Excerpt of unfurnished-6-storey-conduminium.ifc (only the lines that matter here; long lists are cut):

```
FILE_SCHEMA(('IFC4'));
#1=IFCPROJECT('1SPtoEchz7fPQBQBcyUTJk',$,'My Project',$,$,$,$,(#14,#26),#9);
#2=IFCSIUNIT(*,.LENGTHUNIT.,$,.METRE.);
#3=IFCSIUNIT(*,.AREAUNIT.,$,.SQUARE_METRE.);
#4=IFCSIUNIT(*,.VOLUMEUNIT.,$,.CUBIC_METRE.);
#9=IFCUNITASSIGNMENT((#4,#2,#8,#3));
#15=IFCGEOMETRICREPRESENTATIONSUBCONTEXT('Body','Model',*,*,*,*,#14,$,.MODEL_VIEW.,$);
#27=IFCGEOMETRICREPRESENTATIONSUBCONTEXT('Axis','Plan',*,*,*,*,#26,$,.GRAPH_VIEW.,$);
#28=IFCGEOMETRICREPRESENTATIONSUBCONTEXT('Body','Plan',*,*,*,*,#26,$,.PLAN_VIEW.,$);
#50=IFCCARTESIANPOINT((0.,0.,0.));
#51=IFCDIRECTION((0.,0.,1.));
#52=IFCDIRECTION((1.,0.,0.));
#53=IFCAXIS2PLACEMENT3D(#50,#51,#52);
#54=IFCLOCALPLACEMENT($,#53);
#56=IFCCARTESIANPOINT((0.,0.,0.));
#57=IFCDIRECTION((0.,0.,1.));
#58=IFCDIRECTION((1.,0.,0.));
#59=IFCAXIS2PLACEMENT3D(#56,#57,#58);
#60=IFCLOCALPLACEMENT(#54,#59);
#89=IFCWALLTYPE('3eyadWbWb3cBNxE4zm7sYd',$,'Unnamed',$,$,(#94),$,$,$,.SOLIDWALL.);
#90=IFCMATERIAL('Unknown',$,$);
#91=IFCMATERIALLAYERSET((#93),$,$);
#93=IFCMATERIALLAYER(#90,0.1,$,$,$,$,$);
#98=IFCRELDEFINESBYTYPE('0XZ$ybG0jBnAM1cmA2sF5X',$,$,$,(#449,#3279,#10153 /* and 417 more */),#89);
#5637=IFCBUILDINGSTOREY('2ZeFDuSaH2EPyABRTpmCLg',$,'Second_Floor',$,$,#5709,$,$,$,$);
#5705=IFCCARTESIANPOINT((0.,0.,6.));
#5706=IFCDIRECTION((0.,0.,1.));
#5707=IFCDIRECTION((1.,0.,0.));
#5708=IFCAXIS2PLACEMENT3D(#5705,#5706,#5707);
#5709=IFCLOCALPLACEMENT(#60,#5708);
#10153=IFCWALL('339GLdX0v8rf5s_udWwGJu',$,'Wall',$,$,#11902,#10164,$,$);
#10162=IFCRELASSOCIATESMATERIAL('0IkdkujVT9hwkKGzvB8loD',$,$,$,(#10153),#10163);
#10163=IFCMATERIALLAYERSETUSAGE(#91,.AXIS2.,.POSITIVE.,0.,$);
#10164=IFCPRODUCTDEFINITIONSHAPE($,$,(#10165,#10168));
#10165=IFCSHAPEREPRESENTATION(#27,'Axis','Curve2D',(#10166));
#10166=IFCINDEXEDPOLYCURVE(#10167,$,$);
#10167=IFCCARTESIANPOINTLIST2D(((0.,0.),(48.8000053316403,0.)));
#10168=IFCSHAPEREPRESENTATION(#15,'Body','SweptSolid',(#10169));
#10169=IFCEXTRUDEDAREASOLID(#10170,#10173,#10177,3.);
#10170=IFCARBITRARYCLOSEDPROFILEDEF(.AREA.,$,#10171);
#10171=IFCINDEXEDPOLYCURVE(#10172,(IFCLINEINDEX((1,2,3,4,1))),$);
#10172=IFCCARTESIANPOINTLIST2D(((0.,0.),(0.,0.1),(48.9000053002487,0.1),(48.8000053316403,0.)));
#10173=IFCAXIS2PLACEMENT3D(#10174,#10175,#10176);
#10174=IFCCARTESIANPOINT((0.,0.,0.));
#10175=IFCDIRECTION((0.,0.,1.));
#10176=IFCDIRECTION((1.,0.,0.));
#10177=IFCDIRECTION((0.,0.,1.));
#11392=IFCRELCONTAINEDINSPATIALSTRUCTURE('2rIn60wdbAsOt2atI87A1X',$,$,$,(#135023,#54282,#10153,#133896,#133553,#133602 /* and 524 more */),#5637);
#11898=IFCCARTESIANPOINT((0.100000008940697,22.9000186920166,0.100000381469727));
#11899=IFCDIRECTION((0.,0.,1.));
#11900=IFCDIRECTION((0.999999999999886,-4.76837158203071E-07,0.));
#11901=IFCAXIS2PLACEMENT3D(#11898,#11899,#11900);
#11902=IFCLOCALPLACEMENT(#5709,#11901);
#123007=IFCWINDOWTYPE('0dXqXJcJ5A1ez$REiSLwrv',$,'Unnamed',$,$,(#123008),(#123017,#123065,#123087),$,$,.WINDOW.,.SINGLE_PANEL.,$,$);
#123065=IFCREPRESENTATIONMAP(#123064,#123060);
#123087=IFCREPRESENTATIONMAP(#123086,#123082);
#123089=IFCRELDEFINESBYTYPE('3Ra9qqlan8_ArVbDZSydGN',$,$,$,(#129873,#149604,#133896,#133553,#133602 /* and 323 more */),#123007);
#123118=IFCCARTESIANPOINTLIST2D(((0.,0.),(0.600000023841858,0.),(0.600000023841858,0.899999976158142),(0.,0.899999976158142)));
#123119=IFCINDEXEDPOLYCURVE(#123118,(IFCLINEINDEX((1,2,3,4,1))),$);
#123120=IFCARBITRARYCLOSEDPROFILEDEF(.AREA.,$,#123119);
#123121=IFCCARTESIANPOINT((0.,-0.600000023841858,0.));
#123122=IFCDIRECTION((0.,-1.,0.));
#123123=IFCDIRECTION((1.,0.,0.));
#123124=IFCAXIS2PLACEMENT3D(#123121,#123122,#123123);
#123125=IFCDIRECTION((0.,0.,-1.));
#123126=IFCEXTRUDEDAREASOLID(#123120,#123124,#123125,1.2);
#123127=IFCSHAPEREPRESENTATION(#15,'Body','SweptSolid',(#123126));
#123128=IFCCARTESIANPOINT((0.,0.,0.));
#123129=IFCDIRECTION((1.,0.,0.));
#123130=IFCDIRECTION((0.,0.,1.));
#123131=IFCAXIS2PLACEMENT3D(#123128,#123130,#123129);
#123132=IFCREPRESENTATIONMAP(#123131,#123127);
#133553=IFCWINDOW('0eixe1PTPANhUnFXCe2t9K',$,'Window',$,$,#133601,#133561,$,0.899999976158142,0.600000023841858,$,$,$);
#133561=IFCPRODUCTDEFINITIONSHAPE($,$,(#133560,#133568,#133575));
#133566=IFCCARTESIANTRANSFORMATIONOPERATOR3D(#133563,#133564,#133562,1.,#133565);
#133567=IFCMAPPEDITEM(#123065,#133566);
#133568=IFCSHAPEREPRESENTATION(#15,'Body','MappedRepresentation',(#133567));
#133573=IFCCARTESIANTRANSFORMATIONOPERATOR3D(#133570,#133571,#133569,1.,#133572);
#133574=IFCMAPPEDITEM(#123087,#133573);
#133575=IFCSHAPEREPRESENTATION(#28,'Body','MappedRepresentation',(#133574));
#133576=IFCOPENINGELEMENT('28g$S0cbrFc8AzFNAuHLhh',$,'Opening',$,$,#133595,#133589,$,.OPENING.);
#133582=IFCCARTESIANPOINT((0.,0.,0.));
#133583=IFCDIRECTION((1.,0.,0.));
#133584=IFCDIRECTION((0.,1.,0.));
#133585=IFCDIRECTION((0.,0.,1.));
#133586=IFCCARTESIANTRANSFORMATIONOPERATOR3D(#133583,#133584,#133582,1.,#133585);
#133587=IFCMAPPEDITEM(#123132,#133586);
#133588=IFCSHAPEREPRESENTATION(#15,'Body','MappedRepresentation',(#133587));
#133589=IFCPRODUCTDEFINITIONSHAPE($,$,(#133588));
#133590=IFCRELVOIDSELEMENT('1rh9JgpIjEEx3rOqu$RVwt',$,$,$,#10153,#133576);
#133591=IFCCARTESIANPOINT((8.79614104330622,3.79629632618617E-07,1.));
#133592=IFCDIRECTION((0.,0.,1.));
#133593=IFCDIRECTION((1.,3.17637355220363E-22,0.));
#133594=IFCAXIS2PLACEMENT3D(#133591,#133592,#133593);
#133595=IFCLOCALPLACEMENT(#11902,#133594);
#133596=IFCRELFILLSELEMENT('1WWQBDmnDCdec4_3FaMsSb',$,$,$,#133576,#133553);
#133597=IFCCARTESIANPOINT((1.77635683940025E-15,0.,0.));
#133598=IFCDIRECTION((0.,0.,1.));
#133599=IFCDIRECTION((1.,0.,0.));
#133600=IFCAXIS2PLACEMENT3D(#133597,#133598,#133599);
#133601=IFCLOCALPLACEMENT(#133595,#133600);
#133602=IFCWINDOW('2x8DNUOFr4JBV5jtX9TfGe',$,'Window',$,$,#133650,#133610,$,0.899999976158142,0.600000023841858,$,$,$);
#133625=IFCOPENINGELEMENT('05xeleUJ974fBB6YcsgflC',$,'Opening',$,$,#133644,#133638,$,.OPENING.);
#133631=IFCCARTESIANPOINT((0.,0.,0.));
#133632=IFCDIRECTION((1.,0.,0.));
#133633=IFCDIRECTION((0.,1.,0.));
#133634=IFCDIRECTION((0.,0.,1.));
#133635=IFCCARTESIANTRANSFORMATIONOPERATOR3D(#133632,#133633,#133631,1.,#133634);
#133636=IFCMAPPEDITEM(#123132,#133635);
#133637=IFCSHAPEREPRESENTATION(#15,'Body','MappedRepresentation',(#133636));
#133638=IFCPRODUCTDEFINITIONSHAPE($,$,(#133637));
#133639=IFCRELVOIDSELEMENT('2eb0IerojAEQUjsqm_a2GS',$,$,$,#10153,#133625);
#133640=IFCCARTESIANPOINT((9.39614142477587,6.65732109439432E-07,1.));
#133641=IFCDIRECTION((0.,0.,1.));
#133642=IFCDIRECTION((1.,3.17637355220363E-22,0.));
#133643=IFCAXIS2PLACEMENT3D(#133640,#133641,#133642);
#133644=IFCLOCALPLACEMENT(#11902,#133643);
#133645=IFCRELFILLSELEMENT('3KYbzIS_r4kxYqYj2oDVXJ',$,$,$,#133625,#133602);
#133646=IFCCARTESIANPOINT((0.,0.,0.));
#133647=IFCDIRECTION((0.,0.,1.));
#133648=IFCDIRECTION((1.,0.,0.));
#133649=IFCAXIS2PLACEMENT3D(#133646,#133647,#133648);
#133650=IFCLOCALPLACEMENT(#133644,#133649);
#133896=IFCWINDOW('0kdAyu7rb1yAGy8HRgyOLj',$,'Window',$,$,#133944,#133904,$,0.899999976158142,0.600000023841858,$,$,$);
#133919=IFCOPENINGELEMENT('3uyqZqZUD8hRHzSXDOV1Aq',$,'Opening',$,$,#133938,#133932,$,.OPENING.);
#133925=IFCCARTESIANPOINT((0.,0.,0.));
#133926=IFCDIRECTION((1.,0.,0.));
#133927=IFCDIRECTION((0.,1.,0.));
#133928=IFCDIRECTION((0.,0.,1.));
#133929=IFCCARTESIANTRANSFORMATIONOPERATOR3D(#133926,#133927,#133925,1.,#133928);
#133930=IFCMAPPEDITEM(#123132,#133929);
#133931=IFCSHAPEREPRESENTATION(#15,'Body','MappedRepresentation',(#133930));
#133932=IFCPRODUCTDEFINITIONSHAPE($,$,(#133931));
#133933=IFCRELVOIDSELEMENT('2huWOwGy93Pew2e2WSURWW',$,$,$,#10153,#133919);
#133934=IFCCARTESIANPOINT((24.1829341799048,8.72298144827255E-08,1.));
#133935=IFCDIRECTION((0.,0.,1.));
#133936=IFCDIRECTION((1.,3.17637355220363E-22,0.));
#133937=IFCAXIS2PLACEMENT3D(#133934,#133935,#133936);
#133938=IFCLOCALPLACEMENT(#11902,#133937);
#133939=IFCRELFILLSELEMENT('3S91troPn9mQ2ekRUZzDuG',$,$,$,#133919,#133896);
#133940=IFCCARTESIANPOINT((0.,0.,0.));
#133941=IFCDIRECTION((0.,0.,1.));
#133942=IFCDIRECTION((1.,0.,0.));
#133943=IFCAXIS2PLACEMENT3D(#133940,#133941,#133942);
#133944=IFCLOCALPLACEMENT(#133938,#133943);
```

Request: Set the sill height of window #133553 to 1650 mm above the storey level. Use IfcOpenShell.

```python
import numpy as np
import ifcopenshell
import ifcopenshell.api.geometry
import ifcopenshell.geom
import ifcopenshell.util.element
import ifcopenshell.util.placement
import ifcopenshell.util.shape
import ifcopenshell.util.unit

model = ifcopenshell.open("unfurnished-6-storey-conduminium.ifc")
unit_scale = ifcopenshell.util.unit.calculate_unit_scale(model)

window = model.by_guid("0eixe1PTPANhUnFXCe2t9K")
opening = window.FillsVoids[0].RelatingOpeningElement
storey = ifcopenshell.util.element.get_container(window, ifc_class="IfcBuildingStorey")
level = ifcopenshell.util.placement.get_local_placement(storey.ObjectPlacement)[2, 3]

# The opening's origin need not be at the sill, so measure its lowest point.
shape = ifcopenshell.geom.create_shape(ifcopenshell.geom.settings(), opening)
bottom = ifcopenshell.util.shape.get_shape_bottom_elevation(shape, shape.geometry) / unit_scale
dz = level + 1.65 / unit_scale - bottom

shift = np.array([0.0, 0.0, dz])
# The window is placed relative to its opening, so it follows when the opening moves.
matrix = ifcopenshell.util.placement.get_local_placement(opening.ObjectPlacement)
matrix[:3, 3] += shift
ifcopenshell.api.geometry.edit_object_placement(
    model, product=opening, matrix=matrix, is_si=False, should_transform_children=True
)

print(f"moved by {dz * unit_scale:+.3f} m")

model.write("unfurnished-6-storey-conduminium_updated.ifc")
```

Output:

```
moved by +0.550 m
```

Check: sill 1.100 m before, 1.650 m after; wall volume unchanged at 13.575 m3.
